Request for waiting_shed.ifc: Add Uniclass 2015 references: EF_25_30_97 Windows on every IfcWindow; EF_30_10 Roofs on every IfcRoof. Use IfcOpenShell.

First a look at what the model holds.

```python
import ifcopenshell

model = ifcopenshell.open("waiting_shed.ifc")
print(model.schema)
print("classifications:", [c.Name for c in model.by_type("IfcClassification")])
for ifc_class in ("IfcDoor", "IfcRoof", "IfcStair", "IfcWall", "IfcWindow"):
    print(ifc_class, len(model.by_type(ifc_class)))
```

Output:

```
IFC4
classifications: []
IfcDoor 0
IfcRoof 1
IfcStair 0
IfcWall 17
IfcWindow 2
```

```python
import ifcopenshell
import ifcopenshell.api.classification

model = ifcopenshell.open("waiting_shed.ifc")

system = ifcopenshell.api.classification.add_classification(model, classification="Uniclass 2015")

codes = {
    "IfcWindow": ("EF_25_30_97", "Windows"),
    "IfcRoof": ("EF_30_10", "Roofs"),
}
for ifc_class, (code, name) in codes.items():
    products = model.by_type(ifc_class)
    ifcopenshell.api.classification.add_reference(
        model, products=products, classification=system, identification=code, name=name
    )
    print(code, len(products))

model.write("waiting_shed_updated.ifc")
```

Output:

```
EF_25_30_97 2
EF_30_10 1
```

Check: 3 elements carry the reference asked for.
